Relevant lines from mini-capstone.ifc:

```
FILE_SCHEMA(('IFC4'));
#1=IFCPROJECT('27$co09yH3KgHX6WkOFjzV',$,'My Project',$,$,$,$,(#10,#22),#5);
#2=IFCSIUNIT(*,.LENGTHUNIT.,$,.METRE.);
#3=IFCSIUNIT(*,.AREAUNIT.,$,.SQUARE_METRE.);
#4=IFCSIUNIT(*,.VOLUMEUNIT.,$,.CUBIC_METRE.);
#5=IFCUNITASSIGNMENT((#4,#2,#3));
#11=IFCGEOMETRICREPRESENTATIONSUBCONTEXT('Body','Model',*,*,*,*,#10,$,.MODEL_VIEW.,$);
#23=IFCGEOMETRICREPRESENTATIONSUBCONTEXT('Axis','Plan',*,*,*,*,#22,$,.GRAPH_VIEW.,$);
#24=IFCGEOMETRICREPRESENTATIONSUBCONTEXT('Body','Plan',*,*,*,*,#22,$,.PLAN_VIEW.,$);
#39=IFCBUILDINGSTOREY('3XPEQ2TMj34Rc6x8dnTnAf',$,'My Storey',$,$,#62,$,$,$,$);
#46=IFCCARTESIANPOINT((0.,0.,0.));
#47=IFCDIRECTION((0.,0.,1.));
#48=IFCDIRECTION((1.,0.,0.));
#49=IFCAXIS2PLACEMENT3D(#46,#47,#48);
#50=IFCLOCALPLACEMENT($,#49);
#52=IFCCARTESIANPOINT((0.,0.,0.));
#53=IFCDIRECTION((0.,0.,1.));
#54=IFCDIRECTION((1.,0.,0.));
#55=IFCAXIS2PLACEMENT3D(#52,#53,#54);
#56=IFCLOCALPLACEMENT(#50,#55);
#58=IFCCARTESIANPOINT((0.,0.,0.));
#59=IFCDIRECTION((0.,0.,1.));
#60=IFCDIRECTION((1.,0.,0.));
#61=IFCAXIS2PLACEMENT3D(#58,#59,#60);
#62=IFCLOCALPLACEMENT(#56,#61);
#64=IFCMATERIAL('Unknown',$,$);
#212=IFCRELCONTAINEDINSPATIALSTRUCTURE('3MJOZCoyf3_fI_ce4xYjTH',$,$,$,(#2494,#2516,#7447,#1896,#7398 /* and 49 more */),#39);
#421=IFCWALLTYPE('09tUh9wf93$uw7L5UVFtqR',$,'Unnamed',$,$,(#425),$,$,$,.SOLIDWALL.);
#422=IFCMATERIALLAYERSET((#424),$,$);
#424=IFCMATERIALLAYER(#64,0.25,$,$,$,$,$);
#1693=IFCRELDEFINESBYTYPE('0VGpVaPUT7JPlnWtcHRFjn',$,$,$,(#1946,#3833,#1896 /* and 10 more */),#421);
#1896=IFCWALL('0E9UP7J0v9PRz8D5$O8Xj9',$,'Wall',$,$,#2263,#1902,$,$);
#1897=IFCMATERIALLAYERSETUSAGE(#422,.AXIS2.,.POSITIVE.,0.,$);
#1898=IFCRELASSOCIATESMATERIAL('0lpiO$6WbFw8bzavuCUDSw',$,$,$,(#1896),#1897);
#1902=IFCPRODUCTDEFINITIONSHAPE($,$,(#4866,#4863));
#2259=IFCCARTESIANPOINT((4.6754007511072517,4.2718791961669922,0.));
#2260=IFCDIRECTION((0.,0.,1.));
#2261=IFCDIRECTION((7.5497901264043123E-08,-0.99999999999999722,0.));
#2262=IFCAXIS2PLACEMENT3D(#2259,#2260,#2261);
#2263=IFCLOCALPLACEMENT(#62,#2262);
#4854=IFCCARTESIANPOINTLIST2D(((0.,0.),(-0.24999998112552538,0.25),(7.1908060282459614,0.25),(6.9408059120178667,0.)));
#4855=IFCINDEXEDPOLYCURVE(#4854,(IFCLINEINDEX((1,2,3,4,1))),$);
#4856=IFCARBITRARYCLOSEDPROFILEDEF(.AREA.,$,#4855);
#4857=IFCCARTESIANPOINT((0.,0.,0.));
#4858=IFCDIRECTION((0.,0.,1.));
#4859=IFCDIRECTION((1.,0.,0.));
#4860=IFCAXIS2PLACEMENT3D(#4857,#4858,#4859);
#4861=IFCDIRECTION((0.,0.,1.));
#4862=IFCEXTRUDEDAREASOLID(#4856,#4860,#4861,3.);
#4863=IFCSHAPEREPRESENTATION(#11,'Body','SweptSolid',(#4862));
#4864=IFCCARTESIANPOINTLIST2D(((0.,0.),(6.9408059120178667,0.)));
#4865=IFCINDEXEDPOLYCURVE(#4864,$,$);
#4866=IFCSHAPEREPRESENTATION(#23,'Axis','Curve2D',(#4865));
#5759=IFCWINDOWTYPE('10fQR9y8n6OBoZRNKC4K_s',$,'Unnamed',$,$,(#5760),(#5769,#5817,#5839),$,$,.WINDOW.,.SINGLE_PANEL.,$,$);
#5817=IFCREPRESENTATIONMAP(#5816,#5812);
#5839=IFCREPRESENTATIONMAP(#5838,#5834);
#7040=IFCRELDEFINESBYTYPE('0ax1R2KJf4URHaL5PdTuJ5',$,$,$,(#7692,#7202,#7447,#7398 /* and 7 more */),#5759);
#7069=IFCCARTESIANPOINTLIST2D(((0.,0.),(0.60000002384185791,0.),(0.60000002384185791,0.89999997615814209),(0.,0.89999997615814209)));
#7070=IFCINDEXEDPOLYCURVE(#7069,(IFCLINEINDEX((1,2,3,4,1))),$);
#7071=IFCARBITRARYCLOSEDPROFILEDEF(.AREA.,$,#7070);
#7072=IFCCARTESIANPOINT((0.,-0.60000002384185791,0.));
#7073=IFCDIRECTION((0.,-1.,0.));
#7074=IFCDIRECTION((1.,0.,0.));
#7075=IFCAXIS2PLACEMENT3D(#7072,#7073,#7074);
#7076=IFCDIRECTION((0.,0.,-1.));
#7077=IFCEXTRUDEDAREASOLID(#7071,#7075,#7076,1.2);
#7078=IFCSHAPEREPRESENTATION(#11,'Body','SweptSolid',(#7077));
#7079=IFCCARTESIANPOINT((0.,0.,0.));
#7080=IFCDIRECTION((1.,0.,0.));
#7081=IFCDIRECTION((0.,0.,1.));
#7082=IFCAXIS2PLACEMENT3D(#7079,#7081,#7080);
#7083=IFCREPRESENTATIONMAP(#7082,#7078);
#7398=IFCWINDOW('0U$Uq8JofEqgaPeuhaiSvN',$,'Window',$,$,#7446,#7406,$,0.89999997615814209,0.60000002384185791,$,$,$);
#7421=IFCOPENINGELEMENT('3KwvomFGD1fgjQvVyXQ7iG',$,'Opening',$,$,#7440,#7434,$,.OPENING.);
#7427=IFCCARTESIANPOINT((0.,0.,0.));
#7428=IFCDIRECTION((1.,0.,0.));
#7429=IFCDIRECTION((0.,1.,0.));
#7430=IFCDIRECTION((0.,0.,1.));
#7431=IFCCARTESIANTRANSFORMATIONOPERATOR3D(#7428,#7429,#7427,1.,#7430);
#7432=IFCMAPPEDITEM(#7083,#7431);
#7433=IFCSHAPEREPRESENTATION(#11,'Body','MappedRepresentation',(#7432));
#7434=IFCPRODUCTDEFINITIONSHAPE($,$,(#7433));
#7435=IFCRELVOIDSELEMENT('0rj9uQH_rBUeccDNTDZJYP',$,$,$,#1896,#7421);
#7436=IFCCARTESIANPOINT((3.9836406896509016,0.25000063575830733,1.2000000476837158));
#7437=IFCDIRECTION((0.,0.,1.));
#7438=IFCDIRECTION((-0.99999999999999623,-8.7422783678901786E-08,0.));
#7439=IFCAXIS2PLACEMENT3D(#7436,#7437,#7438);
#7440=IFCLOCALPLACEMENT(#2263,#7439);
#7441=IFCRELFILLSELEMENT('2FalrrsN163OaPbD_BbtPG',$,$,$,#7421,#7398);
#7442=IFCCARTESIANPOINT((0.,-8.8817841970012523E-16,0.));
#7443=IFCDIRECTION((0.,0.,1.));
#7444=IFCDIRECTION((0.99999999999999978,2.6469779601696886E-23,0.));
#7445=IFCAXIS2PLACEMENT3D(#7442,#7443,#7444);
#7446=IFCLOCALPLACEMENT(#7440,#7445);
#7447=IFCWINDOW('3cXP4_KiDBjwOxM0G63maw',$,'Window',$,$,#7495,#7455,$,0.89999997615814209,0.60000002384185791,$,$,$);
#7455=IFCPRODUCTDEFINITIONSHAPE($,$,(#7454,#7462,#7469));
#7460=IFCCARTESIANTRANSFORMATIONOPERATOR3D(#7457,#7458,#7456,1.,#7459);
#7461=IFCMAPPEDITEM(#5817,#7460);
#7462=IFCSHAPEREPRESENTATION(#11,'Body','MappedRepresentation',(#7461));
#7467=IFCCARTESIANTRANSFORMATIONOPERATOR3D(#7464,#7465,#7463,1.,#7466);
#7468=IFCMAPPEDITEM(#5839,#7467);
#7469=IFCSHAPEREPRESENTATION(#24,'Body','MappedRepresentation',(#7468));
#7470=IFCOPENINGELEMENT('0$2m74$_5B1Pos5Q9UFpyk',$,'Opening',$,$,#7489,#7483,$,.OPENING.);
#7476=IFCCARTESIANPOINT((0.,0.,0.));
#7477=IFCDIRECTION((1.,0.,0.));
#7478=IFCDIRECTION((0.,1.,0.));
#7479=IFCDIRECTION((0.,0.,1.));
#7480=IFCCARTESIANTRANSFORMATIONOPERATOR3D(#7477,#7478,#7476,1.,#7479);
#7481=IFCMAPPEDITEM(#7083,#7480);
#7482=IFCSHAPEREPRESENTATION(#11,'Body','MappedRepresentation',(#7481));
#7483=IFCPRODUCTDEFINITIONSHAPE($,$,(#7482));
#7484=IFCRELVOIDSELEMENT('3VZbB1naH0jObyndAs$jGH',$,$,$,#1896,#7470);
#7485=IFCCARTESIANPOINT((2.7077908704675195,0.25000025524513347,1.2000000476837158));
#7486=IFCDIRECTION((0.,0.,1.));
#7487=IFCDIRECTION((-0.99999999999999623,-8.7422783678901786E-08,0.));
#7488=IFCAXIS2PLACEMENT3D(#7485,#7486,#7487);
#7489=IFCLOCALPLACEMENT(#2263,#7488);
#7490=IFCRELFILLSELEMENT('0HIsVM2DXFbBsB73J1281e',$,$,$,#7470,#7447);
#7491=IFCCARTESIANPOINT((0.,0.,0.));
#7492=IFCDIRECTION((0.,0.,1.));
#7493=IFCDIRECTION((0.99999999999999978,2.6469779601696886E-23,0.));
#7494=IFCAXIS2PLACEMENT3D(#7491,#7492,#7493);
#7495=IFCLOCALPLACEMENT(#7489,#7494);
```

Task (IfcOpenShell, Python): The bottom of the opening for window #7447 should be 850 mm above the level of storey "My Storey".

```python
import numpy as np
import ifcopenshell
import ifcopenshell.api.geometry
import ifcopenshell.geom
import ifcopenshell.util.element
import ifcopenshell.util.placement
import ifcopenshell.util.shape
import ifcopenshell.util.unit

model = ifcopenshell.open("mini-capstone.ifc")
unit_scale = ifcopenshell.util.unit.calculate_unit_scale(model)

window = model.by_id(7447)
opening = window.FillsVoids[0].RelatingOpeningElement
storey = ifcopenshell.util.element.get_container(window, ifc_class="IfcBuildingStorey")
level = ifcopenshell.util.placement.get_local_placement(storey.ObjectPlacement)[2, 3]

# The opening's origin need not be at the sill, so measure its lowest point.
shape = ifcopenshell.geom.create_shape(ifcopenshell.geom.settings(), opening)
bottom = ifcopenshell.util.shape.get_shape_bottom_elevation(shape, shape.geometry) / unit_scale
dz = level + 0.85 - bottom

shift = np.array([0.0, 0.0, dz])
# The window is placed relative to its opening, so it follows when the opening moves.
matrix = ifcopenshell.util.placement.get_local_placement(opening.ObjectPlacement)
matrix[:3, 3] += shift
ifcopenshell.api.geometry.edit_object_placement(
    model, product=opening, matrix=matrix, is_si=False, should_transform_children=True
)

print(f"moved by {dz * unit_scale:+.3f} m")

model.write("mini-capstone_updated.ifc")
```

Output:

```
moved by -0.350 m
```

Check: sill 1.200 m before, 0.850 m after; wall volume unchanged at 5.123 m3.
